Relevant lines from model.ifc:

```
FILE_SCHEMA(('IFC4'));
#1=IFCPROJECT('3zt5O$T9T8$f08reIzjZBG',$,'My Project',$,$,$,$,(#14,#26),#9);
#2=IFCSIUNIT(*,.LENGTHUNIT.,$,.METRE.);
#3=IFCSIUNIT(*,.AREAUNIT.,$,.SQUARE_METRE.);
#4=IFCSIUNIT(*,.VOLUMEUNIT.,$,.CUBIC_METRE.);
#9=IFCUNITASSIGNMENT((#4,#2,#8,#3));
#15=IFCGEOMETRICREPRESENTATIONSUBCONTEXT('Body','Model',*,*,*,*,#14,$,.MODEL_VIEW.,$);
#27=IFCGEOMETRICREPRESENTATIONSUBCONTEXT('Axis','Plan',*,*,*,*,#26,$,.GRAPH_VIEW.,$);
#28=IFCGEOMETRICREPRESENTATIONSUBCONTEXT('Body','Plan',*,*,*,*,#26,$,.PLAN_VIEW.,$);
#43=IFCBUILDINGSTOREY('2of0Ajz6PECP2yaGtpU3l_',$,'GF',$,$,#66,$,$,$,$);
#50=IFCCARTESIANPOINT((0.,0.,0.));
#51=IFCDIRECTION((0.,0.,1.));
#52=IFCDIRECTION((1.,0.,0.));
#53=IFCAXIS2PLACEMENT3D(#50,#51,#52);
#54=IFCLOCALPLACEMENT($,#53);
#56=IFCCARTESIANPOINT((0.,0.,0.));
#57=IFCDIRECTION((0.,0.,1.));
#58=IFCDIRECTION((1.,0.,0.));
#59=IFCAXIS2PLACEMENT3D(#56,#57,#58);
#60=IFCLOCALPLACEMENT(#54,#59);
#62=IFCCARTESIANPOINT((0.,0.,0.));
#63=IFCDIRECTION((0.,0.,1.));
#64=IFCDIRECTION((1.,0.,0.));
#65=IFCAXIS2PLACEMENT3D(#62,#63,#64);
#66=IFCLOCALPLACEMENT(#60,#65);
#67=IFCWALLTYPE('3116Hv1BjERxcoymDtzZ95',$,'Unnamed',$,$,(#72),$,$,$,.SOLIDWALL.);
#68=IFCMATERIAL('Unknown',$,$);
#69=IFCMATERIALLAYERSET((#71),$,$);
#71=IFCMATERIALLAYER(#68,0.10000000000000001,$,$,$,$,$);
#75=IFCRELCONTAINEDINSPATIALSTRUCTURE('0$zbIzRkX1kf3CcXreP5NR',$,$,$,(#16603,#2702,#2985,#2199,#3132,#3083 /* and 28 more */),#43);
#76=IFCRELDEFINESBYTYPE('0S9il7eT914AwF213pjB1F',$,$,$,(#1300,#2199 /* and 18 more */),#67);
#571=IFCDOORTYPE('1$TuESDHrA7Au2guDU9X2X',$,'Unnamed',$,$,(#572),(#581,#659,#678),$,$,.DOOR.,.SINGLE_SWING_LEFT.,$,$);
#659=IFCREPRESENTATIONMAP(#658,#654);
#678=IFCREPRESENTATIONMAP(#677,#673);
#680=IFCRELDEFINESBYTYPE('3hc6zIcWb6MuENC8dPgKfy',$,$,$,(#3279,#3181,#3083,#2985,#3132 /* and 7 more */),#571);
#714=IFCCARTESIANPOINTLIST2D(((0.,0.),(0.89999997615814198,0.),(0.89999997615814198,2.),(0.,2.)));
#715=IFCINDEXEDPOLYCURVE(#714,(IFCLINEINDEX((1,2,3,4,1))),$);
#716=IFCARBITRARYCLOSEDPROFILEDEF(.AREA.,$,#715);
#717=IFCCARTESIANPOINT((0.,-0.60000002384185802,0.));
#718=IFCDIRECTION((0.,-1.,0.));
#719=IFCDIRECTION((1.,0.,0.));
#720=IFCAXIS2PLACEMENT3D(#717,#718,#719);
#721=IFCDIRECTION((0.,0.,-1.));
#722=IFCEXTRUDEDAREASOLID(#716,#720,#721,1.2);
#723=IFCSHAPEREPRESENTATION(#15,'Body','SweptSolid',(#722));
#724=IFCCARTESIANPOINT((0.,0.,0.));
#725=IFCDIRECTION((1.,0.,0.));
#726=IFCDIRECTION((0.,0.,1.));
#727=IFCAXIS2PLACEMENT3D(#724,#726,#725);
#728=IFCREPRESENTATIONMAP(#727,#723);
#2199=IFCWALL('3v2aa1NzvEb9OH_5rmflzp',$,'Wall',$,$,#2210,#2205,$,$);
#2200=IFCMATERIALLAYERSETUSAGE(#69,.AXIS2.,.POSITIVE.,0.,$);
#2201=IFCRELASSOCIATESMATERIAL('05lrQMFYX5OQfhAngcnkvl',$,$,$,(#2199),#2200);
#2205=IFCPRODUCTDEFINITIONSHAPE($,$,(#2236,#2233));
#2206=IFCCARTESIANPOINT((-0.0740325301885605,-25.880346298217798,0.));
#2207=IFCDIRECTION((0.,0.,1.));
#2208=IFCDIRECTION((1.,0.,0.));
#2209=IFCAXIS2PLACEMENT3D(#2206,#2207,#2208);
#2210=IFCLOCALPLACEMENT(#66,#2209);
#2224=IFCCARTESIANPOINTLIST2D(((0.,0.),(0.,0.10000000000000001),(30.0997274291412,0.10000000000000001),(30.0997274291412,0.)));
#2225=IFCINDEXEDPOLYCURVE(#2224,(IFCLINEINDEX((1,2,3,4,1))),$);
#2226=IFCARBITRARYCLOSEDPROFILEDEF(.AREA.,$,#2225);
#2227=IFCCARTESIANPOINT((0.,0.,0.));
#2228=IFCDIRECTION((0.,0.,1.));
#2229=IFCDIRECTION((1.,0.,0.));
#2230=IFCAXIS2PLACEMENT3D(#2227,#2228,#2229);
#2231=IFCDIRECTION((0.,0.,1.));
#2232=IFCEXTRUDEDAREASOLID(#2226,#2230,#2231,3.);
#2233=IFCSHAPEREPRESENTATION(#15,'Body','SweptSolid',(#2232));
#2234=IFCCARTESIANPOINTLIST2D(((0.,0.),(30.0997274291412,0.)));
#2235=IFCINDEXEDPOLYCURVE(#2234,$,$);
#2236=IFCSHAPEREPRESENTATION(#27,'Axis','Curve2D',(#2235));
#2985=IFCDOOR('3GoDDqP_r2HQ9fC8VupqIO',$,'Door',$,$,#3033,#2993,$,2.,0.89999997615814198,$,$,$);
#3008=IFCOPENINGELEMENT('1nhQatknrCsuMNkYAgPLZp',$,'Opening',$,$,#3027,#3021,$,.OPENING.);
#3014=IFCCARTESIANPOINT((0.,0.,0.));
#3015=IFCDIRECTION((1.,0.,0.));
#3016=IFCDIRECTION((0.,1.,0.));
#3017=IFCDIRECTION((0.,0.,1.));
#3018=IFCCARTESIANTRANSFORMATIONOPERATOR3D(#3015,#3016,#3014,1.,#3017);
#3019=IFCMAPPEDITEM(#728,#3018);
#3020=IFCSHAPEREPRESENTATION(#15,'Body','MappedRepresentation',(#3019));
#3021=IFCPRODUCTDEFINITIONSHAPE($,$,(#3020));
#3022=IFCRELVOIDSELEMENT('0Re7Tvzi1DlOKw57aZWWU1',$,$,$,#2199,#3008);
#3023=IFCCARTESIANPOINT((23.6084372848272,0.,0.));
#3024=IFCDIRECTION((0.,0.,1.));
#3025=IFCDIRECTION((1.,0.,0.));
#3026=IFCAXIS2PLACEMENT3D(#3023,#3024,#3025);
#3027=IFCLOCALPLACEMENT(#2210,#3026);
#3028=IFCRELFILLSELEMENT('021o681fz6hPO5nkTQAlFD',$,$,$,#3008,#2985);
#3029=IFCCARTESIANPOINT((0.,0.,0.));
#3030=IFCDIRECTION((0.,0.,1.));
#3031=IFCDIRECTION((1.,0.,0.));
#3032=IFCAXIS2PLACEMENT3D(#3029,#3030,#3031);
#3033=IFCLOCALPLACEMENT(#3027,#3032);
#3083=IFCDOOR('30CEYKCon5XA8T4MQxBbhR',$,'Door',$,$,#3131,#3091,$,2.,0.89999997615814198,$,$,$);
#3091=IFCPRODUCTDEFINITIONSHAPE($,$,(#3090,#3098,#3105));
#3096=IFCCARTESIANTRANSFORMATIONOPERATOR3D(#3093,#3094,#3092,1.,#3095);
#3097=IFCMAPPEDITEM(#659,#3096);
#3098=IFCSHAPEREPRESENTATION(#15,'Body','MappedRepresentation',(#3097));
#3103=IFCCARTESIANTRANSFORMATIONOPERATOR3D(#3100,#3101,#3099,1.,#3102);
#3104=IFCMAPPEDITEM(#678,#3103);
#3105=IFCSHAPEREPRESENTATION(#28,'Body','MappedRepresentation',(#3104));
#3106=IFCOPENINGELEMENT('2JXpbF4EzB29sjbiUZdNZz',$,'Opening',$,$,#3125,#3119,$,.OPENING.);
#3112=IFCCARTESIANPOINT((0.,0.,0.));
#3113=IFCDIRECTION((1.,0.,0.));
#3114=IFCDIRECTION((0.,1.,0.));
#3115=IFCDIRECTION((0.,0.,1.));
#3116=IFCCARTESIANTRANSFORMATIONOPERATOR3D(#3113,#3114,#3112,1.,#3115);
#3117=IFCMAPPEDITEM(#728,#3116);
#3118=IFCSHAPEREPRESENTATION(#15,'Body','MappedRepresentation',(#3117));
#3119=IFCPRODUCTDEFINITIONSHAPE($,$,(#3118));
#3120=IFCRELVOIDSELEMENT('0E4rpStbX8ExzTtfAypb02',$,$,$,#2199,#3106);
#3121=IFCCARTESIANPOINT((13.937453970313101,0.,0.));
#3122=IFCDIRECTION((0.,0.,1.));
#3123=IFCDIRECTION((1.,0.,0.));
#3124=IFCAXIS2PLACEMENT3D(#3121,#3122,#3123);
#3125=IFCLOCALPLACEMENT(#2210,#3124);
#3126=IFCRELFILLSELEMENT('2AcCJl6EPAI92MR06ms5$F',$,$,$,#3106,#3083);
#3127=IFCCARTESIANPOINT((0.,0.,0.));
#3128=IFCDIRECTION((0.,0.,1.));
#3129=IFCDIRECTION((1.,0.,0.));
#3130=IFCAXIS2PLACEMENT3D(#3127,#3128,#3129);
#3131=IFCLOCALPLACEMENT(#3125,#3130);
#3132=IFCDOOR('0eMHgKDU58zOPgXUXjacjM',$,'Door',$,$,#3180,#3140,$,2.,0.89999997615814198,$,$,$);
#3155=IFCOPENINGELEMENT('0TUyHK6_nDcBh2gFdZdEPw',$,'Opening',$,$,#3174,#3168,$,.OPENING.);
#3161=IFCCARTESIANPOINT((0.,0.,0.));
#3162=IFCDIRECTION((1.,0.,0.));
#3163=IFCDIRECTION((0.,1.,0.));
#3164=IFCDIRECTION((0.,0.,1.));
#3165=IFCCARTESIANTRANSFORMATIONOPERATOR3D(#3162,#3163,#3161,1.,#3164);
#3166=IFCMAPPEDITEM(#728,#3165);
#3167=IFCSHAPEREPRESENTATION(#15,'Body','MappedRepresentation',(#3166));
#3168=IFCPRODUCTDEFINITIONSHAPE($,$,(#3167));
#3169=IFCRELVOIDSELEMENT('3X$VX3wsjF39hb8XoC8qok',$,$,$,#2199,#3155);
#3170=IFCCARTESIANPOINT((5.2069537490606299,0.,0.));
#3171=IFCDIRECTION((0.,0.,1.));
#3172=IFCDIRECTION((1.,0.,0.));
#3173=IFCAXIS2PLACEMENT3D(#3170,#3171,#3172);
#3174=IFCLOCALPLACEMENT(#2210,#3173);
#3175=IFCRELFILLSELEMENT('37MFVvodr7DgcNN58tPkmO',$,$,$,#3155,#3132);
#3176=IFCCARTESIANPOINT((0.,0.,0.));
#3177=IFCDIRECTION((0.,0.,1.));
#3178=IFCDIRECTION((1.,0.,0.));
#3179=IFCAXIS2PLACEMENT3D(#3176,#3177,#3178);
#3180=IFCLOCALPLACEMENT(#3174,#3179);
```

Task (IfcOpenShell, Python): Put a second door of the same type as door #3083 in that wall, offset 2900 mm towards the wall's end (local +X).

```python
import ifcopenshell
import ifcopenshell.api.feature
import ifcopenshell.api.geometry
import ifcopenshell.api.root
import ifcopenshell.geom
import ifcopenshell.util.element
import ifcopenshell.util.placement
import ifcopenshell.util.shape

model = ifcopenshell.open("model.ifc")
settings = ifcopenshell.geom.settings()


def volume(element):
    """Net volume in cubic metres, openings subtracted."""
    shape = ifcopenshell.geom.create_shape(settings, element)
    return ifcopenshell.util.shape.get_volume(shape.geometry)


door = model.by_guid("30CEYKCon5XA8T4MQxBbhR")
opening = door.FillsVoids[0].RelatingOpeningElement
wall = opening.VoidsElements[0].RelatingBuildingElement
before = volume(wall)
shift = ifcopenshell.util.placement.get_local_placement(wall.ObjectPlacement)[:3, 0] * 2.9

# copy_class copies the void relationship, type, container and properties, but no geometry.
new_opening = ifcopenshell.api.root.copy_class(model, product=opening)
new_opening.Representation = ifcopenshell.util.element.copy_deep(
    model, opening.Representation, exclude=["IfcGeometricRepresentationContext", "IfcRepresentationMap"]
)
new_door = ifcopenshell.api.root.copy_class(model, product=door)
new_door.Representation = ifcopenshell.util.element.copy_deep(
    model, door.Representation, exclude=["IfcGeometricRepresentationContext", "IfcRepresentationMap"]
)
ifcopenshell.api.feature.add_filling(model, opening=new_opening, element=new_door)

for old, new in ((opening, new_opening), (door, new_door)):
    matrix = ifcopenshell.util.placement.get_local_placement(old.ObjectPlacement)
    matrix[:3, 3] += shift
    ifcopenshell.api.geometry.edit_object_placement(model, product=new, matrix=matrix, is_si=False)

after = volume(wall)

print(f"wall volume {before:.3f} -> {after:.3f} m3")

model.write("model-out.ifc")
```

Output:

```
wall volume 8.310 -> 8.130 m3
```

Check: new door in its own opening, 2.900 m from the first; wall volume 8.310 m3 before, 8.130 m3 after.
